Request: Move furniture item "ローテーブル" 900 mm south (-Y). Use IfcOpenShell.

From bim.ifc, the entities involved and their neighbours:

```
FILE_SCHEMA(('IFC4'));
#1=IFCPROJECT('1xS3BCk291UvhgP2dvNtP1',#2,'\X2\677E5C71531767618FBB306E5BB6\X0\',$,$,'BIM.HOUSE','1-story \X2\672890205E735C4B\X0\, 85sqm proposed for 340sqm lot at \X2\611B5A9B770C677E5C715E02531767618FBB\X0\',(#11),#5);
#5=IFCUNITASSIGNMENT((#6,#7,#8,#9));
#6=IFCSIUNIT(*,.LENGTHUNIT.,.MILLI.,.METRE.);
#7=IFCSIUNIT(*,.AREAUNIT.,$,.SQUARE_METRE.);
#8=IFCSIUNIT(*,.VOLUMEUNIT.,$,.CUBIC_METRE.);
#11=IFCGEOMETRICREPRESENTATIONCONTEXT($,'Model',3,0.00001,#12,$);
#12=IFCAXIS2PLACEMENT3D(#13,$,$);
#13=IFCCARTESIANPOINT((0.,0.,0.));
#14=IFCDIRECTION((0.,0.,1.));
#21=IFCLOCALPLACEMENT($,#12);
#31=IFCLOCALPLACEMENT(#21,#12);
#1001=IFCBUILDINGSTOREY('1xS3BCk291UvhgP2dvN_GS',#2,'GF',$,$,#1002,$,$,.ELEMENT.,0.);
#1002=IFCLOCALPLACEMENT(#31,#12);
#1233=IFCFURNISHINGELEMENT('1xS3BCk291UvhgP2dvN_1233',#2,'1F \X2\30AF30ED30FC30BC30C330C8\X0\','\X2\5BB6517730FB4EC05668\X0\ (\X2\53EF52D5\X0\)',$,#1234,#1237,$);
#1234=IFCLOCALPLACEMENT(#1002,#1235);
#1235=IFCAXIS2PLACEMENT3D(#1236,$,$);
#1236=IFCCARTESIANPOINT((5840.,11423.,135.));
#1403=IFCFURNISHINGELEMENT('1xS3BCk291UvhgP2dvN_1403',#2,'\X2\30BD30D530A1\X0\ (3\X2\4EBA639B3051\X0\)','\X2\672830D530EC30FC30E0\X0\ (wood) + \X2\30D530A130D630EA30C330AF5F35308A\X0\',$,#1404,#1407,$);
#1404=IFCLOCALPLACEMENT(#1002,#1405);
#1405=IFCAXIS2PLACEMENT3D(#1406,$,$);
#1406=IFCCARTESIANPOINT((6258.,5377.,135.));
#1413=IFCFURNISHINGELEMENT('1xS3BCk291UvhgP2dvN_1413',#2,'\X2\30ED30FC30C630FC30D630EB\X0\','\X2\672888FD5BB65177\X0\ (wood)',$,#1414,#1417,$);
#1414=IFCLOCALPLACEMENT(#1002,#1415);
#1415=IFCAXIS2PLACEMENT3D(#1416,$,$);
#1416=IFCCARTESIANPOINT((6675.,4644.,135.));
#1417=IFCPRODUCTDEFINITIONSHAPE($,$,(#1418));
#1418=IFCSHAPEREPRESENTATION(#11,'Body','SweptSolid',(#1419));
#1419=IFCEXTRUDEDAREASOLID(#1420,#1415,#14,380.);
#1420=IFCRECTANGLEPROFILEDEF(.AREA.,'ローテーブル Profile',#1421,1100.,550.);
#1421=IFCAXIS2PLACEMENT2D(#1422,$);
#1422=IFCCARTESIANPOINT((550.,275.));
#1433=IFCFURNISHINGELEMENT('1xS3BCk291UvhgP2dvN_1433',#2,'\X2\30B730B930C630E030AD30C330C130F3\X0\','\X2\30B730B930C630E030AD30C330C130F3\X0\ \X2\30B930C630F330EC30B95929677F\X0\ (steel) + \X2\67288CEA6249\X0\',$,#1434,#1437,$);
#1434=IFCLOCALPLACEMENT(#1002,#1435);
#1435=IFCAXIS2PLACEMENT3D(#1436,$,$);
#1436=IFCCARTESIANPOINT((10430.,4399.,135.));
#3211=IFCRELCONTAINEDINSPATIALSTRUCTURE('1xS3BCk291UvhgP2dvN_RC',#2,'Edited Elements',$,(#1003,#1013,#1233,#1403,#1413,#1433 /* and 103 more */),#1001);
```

```python
import ifcopenshell
import ifcopenshell.api.geometry
import ifcopenshell.util.placement
import ifcopenshell.util.unit

model = ifcopenshell.open("bim.ifc")
unit_scale = ifcopenshell.util.unit.calculate_unit_scale(model)

item = model.by_guid("1xS3BCk291UvhgP2dvN_1413")
matrix = ifcopenshell.util.placement.get_local_placement(item.ObjectPlacement)
matrix[1, 3] -= 0.9 / unit_scale
ifcopenshell.api.geometry.edit_object_placement(model, product=item, matrix=matrix, is_si=False)

print(ifcopenshell.util.placement.get_local_placement(item.ObjectPlacement).round(3) + 0.0)

model.write("bim_edited.ifc")
```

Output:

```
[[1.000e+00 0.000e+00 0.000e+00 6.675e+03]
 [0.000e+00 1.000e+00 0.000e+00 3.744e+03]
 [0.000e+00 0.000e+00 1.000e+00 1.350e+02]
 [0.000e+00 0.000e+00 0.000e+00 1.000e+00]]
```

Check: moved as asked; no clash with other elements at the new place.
